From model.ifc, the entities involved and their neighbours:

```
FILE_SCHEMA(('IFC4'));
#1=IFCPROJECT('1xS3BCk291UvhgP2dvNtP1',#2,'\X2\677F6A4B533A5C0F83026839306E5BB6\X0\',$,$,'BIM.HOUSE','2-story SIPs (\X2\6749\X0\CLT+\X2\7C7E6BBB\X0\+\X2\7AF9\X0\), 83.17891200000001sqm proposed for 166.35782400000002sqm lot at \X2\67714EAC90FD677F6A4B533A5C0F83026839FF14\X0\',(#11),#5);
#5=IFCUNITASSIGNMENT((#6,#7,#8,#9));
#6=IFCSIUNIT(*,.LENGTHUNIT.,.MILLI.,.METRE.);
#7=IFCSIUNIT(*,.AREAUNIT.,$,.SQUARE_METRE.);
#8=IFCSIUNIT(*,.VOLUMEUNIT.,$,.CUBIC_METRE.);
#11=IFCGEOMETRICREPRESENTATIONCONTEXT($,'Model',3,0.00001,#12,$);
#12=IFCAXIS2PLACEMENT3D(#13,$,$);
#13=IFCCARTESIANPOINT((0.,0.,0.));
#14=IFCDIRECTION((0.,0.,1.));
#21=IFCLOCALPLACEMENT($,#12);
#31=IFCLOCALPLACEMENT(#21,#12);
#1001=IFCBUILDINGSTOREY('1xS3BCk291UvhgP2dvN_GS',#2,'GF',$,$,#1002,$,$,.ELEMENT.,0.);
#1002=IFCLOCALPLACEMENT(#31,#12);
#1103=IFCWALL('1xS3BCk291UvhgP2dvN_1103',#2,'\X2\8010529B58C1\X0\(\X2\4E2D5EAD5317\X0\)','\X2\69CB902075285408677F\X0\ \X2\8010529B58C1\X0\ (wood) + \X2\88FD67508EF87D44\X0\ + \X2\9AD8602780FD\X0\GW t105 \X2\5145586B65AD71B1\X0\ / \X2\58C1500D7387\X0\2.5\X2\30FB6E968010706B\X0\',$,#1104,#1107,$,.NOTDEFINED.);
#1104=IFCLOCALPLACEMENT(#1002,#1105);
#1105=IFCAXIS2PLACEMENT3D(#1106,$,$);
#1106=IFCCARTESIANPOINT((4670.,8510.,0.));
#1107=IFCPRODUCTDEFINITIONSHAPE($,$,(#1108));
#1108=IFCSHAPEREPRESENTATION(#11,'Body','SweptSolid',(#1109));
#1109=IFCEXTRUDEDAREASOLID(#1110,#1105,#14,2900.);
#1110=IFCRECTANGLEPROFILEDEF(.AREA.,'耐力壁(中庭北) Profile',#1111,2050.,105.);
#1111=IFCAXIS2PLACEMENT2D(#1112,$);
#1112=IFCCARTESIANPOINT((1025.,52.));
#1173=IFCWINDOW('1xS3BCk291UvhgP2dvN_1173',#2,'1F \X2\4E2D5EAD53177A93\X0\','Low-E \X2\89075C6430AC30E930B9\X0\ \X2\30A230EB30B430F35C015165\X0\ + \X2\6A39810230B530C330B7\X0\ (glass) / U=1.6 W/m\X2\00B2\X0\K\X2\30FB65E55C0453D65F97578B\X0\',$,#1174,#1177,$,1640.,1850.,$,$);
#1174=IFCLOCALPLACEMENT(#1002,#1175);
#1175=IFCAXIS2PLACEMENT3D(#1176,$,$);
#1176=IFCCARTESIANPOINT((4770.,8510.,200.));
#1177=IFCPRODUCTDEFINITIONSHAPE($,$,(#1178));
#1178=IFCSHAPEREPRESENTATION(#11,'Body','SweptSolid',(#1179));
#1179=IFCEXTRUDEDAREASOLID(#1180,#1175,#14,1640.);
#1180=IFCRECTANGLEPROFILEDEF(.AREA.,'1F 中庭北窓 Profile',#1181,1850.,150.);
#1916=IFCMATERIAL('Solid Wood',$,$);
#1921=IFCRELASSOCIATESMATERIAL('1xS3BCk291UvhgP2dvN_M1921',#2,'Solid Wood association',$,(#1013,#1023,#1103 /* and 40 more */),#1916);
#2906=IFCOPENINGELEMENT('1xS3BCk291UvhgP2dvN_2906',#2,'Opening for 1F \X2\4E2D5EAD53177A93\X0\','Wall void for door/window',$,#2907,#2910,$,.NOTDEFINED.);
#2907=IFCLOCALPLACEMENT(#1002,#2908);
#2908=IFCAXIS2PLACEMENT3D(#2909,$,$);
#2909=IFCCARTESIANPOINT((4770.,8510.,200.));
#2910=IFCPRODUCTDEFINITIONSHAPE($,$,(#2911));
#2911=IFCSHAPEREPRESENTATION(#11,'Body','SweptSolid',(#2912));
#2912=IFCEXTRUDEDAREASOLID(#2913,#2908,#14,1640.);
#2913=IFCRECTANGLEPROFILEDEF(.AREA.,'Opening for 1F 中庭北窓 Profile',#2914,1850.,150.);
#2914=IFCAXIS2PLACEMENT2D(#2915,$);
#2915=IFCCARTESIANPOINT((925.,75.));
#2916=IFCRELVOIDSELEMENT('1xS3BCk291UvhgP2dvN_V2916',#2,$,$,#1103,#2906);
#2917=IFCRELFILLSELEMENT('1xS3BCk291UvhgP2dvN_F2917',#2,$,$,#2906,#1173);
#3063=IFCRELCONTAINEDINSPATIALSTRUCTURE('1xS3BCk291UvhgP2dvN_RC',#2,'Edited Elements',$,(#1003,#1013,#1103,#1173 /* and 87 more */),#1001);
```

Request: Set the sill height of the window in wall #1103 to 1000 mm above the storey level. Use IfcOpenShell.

```python
import numpy as np
import ifcopenshell
import ifcopenshell.api.geometry
import ifcopenshell.geom
import ifcopenshell.util.element
import ifcopenshell.util.placement
import ifcopenshell.util.shape
import ifcopenshell.util.unit

model = ifcopenshell.open("model.ifc")
unit_scale = ifcopenshell.util.unit.calculate_unit_scale(model)

window = model.by_id(1173)
opening = window.FillsVoids[0].RelatingOpeningElement
storey = ifcopenshell.util.element.get_container(window, ifc_class="IfcBuildingStorey")
level = ifcopenshell.util.placement.get_local_placement(storey.ObjectPlacement)[2, 3]

# The opening's origin need not be at the sill, so measure its lowest point.
shape = ifcopenshell.geom.create_shape(ifcopenshell.geom.settings(), opening)
bottom = ifcopenshell.util.shape.get_shape_bottom_elevation(shape, shape.geometry) / unit_scale
dz = level + 1000.0 - bottom

shift = np.array([0.0, 0.0, dz])
# The window is not placed relative to its opening, so move both.
for product in (opening, window):
    matrix = ifcopenshell.util.placement.get_local_placement(product.ObjectPlacement)
    matrix[:3, 3] += shift
    ifcopenshell.api.geometry.edit_object_placement(model, product=product, matrix=matrix, is_si=False)

print(f"moved by {dz * unit_scale:+.3f} m")

model.write("model_v2.ifc")
```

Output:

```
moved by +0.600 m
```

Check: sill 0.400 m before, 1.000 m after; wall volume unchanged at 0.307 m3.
